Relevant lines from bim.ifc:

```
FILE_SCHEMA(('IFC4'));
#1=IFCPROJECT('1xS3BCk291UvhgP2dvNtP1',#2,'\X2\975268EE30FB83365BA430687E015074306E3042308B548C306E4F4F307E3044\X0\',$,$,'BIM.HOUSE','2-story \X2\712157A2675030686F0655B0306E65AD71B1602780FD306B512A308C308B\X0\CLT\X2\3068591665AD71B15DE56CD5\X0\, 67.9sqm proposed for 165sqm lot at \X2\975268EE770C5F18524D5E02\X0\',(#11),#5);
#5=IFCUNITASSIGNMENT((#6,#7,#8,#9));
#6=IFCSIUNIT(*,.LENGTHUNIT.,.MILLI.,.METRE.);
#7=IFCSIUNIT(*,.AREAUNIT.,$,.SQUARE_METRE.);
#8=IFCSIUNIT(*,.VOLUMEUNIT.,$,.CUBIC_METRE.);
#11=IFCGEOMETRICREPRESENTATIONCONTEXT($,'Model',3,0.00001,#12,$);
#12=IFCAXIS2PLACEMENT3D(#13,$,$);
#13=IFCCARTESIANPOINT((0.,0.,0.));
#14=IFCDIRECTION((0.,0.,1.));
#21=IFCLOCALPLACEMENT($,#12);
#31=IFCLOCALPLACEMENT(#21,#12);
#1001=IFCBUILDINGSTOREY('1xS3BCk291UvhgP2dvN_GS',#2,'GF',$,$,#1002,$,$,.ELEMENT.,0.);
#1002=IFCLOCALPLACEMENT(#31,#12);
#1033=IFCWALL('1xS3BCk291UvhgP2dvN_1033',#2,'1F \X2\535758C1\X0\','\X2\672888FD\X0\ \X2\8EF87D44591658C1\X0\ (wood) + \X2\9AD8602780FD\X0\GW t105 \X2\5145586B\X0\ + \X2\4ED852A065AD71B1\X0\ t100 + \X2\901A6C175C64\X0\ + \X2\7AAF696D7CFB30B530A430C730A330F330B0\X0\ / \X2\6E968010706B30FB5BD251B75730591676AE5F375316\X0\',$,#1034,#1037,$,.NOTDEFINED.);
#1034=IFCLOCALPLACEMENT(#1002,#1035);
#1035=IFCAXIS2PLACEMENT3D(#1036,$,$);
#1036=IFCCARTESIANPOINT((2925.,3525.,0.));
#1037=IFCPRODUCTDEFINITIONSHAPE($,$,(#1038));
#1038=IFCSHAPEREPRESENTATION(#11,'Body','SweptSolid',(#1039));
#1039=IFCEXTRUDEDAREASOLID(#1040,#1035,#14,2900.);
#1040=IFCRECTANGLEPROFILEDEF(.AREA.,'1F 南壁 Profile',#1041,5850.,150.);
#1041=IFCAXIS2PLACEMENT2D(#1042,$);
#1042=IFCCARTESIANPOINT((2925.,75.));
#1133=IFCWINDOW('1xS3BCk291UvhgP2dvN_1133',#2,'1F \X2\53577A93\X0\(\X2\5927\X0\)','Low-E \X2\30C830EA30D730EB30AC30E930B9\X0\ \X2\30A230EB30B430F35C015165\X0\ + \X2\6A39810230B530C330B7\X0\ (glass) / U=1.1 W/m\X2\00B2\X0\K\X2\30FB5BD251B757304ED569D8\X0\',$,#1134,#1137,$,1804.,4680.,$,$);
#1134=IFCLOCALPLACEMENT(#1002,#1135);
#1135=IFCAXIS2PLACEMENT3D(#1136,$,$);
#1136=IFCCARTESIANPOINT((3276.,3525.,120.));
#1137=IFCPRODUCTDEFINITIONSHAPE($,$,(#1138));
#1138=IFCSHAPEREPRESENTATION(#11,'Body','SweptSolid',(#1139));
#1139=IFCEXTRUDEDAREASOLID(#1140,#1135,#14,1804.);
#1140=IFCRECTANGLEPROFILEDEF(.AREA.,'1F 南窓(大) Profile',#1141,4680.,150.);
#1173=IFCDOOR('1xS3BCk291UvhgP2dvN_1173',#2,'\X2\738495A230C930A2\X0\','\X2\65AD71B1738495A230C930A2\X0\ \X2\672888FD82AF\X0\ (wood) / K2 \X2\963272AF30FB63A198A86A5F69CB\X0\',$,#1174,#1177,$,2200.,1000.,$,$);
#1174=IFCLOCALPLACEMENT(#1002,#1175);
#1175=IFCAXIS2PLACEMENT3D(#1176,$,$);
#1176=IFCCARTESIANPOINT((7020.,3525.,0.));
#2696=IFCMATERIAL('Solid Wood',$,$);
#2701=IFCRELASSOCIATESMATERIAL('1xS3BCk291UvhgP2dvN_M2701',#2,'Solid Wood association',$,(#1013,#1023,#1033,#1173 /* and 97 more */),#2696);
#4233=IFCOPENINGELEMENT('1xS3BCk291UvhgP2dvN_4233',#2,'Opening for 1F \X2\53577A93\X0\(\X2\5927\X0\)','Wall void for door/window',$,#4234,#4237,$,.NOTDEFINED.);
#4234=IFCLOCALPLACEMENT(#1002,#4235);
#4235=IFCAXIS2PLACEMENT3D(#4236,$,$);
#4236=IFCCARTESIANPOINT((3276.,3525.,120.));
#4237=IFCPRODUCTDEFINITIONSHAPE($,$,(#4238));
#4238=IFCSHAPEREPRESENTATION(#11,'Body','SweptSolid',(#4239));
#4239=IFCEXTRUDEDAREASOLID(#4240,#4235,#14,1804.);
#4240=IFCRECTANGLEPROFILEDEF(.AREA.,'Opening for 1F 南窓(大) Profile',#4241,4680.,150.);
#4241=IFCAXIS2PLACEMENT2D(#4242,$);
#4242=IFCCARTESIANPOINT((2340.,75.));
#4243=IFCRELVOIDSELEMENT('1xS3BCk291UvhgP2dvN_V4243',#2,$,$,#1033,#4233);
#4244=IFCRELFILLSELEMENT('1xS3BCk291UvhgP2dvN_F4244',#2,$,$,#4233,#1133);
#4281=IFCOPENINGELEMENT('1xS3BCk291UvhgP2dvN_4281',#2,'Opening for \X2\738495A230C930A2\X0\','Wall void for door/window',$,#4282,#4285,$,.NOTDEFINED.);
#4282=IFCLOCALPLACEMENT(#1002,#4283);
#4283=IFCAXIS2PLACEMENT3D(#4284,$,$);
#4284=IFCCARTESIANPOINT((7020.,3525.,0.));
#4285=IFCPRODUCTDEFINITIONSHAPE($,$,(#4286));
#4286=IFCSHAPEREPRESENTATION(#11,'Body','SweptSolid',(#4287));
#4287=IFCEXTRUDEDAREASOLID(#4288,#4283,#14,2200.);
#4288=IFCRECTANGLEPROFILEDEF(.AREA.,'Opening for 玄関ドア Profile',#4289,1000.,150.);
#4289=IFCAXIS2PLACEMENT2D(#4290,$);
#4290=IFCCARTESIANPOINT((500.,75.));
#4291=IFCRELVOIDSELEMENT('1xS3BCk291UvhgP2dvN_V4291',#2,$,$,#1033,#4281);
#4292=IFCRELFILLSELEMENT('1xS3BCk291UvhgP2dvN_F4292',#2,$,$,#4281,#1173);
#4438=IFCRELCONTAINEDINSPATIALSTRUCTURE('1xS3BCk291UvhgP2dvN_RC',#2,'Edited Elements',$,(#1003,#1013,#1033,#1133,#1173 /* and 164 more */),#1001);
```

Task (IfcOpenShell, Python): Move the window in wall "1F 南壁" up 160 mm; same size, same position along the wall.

```python
import numpy as np
import ifcopenshell
import ifcopenshell.api.geometry
import ifcopenshell.util.placement
import ifcopenshell.util.unit

model = ifcopenshell.open("bim.ifc")
unit_scale = ifcopenshell.util.unit.calculate_unit_scale(model)

window = model.by_guid("1xS3BCk291UvhgP2dvN_1133")
opening = window.FillsVoids[0].RelatingOpeningElement
dz = 0.16 / unit_scale

shift = np.array([0.0, 0.0, dz])
# The window is not placed relative to its opening, so move both.
for product in (opening, window):
    matrix = ifcopenshell.util.placement.get_local_placement(product.ObjectPlacement)
    matrix[:3, 3] += shift
    ifcopenshell.api.geometry.edit_object_placement(model, product=product, matrix=matrix, is_si=False)

print(f"moved by {dz * unit_scale:+.3f} m")

model.write("bim-out.ifc")
```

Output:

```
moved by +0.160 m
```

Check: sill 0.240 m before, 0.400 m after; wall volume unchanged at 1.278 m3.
